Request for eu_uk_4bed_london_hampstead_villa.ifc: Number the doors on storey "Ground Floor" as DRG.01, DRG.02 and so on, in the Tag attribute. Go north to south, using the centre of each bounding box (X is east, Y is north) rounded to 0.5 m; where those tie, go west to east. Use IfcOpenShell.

First a look at what the model holds.

```python
import ifcopenshell
import ifcopenshell.util.element
import ifcopenshell.util.placement

model = ifcopenshell.open("eu_uk_4bed_london_hampstead_villa.ifc")
print(model.schema)
storey = next(s for s in model.by_type("IfcBuildingStorey") if s.Name == "Ground Floor")
doors = [e for e in ifcopenshell.util.element.get_decomposition(storey) if e.is_a("IfcDoor")]
for e in sorted(doors, key=lambda e: e.id()):
    origin = ifcopenshell.util.placement.get_local_placement(e.ObjectPlacement)[:3, 3]
    print(e.id(), e.Tag, e.Name, origin.round(2) + 0.0, sep=" | ")
```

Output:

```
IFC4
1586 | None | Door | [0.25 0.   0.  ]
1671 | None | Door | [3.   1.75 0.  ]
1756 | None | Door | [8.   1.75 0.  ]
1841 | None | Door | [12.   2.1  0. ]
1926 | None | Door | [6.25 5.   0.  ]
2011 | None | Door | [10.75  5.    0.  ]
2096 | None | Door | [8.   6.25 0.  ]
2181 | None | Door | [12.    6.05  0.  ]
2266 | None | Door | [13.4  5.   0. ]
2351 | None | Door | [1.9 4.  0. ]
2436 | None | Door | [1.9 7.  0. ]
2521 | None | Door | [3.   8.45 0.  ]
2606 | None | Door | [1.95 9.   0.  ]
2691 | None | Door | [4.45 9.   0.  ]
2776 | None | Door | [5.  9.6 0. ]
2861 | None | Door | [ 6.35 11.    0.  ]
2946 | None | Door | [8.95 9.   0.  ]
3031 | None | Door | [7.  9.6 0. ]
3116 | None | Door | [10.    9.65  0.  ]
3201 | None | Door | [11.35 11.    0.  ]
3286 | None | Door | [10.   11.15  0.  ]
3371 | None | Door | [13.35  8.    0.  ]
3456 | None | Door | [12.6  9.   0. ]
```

```python
import ifcopenshell
import ifcopenshell.geom
import ifcopenshell.util.element
import ifcopenshell.util.shape

model = ifcopenshell.open("eu_uk_4bed_london_hampstead_villa.ifc")
settings = ifcopenshell.geom.settings()
settings.set("use-world-coords", True)


def centre(element):
    shape = ifcopenshell.geom.create_shape(settings, element)
    return ifcopenshell.util.shape.get_bbox_centroid(shape.geometry)


storey = next(s for s in model.by_type("IfcBuildingStorey") if s.Name == "Ground Floor")
doors = [e for e in ifcopenshell.util.element.get_decomposition(storey) if e.is_a("IfcDoor")]

# Insertion points can sit at a corner or the storey origin, so sort by the geometry (in metres).
centres = {e: centre(e) for e in doors}
doors.sort(key=lambda e: (-round(centres[e][1] / 0.5), centres[e][0]))

for i, e in enumerate(doors, start=1):
    number = f"DRG.{i:02d}"
    e.Tag = number
    print(e.id(), number)

model.write("eu_uk_4bed_london_hampstead_villa_updated.ifc")
```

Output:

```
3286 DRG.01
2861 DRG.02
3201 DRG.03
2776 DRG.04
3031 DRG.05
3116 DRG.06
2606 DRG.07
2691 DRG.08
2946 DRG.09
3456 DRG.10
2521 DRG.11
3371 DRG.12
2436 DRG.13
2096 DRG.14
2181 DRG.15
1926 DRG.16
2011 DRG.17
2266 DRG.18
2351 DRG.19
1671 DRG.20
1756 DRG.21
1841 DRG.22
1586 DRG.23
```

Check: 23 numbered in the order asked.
